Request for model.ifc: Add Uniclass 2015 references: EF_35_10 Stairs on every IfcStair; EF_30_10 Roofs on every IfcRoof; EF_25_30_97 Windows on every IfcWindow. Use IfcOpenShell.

First a look at what the model holds.

```python
import ifcopenshell

model = ifcopenshell.open("model.ifc")
print(model.schema)
print("classifications:", [c.Name for c in model.by_type("IfcClassification")])
for ifc_class in ("IfcDoor", "IfcRoof", "IfcStair", "IfcWall", "IfcWindow"):
    print(ifc_class, len(model.by_type(ifc_class)))
```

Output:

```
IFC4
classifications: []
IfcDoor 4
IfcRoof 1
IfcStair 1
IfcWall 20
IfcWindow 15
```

```python
import ifcopenshell
import ifcopenshell.api.classification

model = ifcopenshell.open("model.ifc")

system = ifcopenshell.api.classification.add_classification(model, classification="Uniclass 2015")

codes = {
    "IfcStair": ("EF_35_10", "Stairs"),
    "IfcRoof": ("EF_30_10", "Roofs"),
    "IfcWindow": ("EF_25_30_97", "Windows"),
}
for ifc_class, (code, name) in codes.items():
    products = model.by_type(ifc_class)
    ifcopenshell.api.classification.add_reference(
        model, products=products, classification=system, identification=code, name=name
    )
    print(code, len(products))

model.write("model_v2.ifc")
```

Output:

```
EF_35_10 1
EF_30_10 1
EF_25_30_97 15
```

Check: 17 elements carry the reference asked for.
